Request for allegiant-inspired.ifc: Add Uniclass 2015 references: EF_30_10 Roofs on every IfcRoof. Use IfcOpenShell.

First a look at what the model holds.

```python
import ifcopenshell

model = ifcopenshell.open("allegiant-inspired.ifc")
print(model.schema)
print("classifications:", [c.Name for c in model.by_type("IfcClassification")])
for ifc_class in ("IfcDoor", "IfcRoof", "IfcStair", "IfcWall", "IfcWindow"):
    print(ifc_class, len(model.by_type(ifc_class)))
```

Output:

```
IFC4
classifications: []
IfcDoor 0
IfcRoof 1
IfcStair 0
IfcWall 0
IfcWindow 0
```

```python
import ifcopenshell
import ifcopenshell.api.classification

model = ifcopenshell.open("allegiant-inspired.ifc")

system = ifcopenshell.api.classification.add_classification(model, classification="Uniclass 2015")

codes = {
    "IfcRoof": ("EF_30_10", "Roofs"),
}
for ifc_class, (code, name) in codes.items():
    products = model.by_type(ifc_class)
    ifcopenshell.api.classification.add_reference(
        model, products=products, classification=system, identification=code, name=name
    )
    print(code, len(products))

model.write("allegiant-inspired-out.ifc")
```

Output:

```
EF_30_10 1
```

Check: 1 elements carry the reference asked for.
